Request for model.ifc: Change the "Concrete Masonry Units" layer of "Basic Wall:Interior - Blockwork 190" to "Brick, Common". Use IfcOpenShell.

First a look at what the model holds.

```python
import ifcopenshell
import ifcopenshell.util.element

model = ifcopenshell.open("model.ifc")
print(model.schema)
for layer_set in model.by_type("IfcMaterialLayerSet"):
    if layer_set.LayerSetName == "Basic Wall:Interior - Blockwork 190":
        for layer in layer_set.MaterialLayers:
            print(layer.id(), layer.Material and layer.Material.Name, layer.LayerThickness, sep=" | ")
        print(len(ifcopenshell.util.element.get_elements_by_material(model, layer_set)), "elements and types use it")
print(sorted(m.Name for m in model.by_type("IfcMaterial") if m.Name)[:60])
```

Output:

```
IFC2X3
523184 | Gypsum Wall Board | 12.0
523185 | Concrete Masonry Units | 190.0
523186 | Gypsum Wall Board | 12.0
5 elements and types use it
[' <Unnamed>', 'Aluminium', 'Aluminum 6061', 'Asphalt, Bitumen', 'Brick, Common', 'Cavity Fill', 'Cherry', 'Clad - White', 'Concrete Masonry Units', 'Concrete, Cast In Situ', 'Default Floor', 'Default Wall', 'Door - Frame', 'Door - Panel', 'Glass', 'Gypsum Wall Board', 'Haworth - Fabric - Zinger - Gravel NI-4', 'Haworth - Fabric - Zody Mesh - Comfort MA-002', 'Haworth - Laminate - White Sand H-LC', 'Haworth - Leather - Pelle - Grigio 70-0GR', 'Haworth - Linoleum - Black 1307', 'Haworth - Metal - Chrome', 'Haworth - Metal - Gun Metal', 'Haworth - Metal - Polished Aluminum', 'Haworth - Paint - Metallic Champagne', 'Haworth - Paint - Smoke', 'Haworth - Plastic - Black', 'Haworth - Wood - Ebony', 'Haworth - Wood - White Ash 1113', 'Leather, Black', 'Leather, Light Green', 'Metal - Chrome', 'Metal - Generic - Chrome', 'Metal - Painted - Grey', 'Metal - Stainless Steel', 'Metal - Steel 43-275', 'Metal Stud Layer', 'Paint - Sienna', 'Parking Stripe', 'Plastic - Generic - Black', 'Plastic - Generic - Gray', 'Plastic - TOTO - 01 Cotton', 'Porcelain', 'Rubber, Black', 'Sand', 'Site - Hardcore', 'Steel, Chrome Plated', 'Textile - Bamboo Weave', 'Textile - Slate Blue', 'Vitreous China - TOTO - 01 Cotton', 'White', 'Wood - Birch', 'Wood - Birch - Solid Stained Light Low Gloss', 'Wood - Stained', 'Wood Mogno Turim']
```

```python
import ifcopenshell
import ifcopenshell.api.material

model = ifcopenshell.open("model.ifc")

layer_set = next(s for s in model.by_type("IfcMaterialLayerSet") if s.LayerSetName == "Basic Wall:Interior - Blockwork 190")
layer = next(l for l in layer_set.MaterialLayers if l.Material and l.Material.Name == "Concrete Masonry Units")
material = next(m for m in model.by_type("IfcMaterial") if m.Name == "Brick, Common")

# Point this one layer at the other material; renaming the old one would change it everywhere.
ifcopenshell.api.material.edit_layer(model, layer=layer, attributes={}, material=material)

print([l.Material.Name if l.Material else None for l in layer_set.MaterialLayers])

model.write("model-out.ifc")
```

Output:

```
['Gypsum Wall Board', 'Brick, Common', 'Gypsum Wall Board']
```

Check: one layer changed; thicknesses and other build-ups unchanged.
